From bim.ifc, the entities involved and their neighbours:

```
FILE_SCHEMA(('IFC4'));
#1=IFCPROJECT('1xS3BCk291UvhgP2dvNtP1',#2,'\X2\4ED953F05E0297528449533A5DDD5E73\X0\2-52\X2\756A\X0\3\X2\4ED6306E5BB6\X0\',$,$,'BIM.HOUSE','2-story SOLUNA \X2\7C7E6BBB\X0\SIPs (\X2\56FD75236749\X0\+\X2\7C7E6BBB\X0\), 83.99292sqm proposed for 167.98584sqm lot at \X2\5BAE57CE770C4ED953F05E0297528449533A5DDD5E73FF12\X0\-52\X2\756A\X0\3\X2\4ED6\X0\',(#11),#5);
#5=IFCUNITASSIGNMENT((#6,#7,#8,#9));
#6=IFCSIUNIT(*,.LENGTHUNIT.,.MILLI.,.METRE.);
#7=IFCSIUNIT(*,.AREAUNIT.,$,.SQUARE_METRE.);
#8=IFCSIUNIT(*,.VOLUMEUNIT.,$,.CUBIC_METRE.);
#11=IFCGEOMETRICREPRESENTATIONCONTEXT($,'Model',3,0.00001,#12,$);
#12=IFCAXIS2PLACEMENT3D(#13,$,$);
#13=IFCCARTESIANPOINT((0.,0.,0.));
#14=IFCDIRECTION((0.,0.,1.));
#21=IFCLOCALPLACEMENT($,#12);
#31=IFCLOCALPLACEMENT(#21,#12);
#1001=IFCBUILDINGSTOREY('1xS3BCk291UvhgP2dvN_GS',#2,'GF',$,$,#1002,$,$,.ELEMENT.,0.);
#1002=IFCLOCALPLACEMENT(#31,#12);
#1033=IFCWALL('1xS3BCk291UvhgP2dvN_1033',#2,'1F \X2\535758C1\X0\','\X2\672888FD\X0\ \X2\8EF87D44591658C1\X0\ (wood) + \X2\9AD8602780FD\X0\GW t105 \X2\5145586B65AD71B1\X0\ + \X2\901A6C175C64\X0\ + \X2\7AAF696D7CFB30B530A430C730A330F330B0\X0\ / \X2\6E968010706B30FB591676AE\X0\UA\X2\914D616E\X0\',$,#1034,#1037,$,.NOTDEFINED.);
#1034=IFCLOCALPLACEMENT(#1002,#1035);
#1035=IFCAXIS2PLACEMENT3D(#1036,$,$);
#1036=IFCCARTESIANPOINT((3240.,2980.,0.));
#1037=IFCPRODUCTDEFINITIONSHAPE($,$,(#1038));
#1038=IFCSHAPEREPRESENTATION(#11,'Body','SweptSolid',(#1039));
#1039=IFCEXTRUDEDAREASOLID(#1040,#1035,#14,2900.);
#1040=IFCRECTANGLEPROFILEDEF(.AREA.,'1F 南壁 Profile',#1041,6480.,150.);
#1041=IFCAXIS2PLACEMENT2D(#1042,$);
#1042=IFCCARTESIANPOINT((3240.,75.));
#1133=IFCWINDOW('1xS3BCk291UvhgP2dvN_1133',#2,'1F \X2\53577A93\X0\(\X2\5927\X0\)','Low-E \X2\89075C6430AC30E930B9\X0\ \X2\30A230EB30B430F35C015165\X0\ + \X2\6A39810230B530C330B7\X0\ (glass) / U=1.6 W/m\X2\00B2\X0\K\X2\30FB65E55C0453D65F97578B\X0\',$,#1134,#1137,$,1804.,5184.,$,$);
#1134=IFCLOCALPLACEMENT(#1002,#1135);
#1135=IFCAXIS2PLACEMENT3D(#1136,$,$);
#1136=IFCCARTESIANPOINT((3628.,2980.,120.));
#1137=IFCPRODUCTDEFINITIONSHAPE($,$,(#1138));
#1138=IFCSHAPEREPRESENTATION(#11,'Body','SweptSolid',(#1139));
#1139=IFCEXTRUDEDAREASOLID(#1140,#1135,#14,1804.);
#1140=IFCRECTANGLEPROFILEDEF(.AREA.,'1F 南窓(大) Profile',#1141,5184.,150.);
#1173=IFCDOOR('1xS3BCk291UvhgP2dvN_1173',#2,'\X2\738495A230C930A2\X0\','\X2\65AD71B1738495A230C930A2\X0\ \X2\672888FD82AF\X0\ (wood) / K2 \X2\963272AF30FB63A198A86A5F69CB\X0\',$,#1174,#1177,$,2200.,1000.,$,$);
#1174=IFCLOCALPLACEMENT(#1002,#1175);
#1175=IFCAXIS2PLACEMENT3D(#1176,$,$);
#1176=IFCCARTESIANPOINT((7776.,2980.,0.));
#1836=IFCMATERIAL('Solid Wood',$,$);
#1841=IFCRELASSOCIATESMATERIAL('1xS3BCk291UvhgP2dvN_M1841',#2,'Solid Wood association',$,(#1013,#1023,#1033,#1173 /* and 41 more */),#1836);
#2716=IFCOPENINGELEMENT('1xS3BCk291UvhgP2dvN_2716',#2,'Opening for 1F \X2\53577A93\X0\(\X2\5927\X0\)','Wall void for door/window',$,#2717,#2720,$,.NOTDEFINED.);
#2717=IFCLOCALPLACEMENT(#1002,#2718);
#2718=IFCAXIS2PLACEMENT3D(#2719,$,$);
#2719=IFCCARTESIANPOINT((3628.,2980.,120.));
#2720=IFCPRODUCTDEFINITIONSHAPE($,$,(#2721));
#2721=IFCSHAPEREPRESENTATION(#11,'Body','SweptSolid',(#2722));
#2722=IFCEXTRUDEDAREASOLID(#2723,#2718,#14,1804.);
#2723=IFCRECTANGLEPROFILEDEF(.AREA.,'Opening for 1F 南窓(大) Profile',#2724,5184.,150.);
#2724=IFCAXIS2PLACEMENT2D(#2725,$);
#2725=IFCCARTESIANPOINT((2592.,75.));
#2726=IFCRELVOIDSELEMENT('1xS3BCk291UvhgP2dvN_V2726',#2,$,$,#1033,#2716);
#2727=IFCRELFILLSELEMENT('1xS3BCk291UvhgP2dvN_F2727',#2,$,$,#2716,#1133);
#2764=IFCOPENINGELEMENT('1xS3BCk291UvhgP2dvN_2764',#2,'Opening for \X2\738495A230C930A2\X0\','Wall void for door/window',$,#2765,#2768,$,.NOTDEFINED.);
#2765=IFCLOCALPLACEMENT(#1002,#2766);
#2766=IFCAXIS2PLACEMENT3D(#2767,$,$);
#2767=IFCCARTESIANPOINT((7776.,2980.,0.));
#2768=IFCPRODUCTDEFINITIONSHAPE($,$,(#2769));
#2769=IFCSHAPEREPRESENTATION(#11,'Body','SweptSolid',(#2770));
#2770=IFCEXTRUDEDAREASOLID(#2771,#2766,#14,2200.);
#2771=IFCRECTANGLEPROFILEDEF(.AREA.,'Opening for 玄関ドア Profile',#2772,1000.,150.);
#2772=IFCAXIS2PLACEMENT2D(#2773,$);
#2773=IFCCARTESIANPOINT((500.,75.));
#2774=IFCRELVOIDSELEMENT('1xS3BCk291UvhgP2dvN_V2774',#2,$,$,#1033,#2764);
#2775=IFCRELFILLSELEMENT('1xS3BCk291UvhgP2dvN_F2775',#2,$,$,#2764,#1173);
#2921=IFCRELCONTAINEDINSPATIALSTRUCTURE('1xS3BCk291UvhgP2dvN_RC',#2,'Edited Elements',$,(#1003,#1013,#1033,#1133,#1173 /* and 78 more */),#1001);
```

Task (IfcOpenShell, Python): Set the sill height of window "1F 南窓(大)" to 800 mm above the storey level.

```python
import numpy as np
import ifcopenshell
import ifcopenshell.api.geometry
import ifcopenshell.geom
import ifcopenshell.util.element
import ifcopenshell.util.placement
import ifcopenshell.util.shape
import ifcopenshell.util.unit

model = ifcopenshell.open("bim.ifc")
unit_scale = ifcopenshell.util.unit.calculate_unit_scale(model)

window = model.by_guid("1xS3BCk291UvhgP2dvN_1133")
opening = window.FillsVoids[0].RelatingOpeningElement
storey = ifcopenshell.util.element.get_container(window, ifc_class="IfcBuildingStorey")
level = ifcopenshell.util.placement.get_local_placement(storey.ObjectPlacement)[2, 3]

# The opening's origin need not be at the sill, so measure its lowest point.
shape = ifcopenshell.geom.create_shape(ifcopenshell.geom.settings(), opening)
bottom = ifcopenshell.util.shape.get_shape_bottom_elevation(shape, shape.geometry) / unit_scale
dz = level + 800.0 - bottom

shift = np.array([0.0, 0.0, dz])
# The window is not placed relative to its opening, so move both.
for product in (opening, window):
    matrix = ifcopenshell.util.placement.get_local_placement(product.ObjectPlacement)
    matrix[:3, 3] += shift
    ifcopenshell.api.geometry.edit_object_placement(model, product=product, matrix=matrix, is_si=False)

print(f"moved by {dz * unit_scale:+.3f} m")

model.write("bim_rev.ifc")
```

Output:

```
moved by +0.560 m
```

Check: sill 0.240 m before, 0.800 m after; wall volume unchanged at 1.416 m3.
